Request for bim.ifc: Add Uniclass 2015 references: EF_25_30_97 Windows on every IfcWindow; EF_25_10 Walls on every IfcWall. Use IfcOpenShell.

First a look at what the model holds.

```python
import ifcopenshell

model = ifcopenshell.open("bim.ifc")
print(model.schema)
print("classifications:", [c.Name for c in model.by_type("IfcClassification")])
for ifc_class in ("IfcDoor", "IfcRoof", "IfcStair", "IfcWall", "IfcWindow"):
    print(ifc_class, len(model.by_type(ifc_class)))
```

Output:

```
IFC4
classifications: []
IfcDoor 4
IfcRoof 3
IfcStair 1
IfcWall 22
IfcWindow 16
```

```python
import ifcopenshell
import ifcopenshell.api.classification

model = ifcopenshell.open("bim.ifc")

system = ifcopenshell.api.classification.add_classification(model, classification="Uniclass 2015")

codes = {
    "IfcWindow": ("EF_25_30_97", "Windows"),
    "IfcWall": ("EF_25_10", "Walls"),
}
for ifc_class, (code, name) in codes.items():
    products = model.by_type(ifc_class)
    ifcopenshell.api.classification.add_reference(
        model, products=products, classification=system, identification=code, name=name
    )
    print(code, len(products))

model.write("bim_v2.ifc")
```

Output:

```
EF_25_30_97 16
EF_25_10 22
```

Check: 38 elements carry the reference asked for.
